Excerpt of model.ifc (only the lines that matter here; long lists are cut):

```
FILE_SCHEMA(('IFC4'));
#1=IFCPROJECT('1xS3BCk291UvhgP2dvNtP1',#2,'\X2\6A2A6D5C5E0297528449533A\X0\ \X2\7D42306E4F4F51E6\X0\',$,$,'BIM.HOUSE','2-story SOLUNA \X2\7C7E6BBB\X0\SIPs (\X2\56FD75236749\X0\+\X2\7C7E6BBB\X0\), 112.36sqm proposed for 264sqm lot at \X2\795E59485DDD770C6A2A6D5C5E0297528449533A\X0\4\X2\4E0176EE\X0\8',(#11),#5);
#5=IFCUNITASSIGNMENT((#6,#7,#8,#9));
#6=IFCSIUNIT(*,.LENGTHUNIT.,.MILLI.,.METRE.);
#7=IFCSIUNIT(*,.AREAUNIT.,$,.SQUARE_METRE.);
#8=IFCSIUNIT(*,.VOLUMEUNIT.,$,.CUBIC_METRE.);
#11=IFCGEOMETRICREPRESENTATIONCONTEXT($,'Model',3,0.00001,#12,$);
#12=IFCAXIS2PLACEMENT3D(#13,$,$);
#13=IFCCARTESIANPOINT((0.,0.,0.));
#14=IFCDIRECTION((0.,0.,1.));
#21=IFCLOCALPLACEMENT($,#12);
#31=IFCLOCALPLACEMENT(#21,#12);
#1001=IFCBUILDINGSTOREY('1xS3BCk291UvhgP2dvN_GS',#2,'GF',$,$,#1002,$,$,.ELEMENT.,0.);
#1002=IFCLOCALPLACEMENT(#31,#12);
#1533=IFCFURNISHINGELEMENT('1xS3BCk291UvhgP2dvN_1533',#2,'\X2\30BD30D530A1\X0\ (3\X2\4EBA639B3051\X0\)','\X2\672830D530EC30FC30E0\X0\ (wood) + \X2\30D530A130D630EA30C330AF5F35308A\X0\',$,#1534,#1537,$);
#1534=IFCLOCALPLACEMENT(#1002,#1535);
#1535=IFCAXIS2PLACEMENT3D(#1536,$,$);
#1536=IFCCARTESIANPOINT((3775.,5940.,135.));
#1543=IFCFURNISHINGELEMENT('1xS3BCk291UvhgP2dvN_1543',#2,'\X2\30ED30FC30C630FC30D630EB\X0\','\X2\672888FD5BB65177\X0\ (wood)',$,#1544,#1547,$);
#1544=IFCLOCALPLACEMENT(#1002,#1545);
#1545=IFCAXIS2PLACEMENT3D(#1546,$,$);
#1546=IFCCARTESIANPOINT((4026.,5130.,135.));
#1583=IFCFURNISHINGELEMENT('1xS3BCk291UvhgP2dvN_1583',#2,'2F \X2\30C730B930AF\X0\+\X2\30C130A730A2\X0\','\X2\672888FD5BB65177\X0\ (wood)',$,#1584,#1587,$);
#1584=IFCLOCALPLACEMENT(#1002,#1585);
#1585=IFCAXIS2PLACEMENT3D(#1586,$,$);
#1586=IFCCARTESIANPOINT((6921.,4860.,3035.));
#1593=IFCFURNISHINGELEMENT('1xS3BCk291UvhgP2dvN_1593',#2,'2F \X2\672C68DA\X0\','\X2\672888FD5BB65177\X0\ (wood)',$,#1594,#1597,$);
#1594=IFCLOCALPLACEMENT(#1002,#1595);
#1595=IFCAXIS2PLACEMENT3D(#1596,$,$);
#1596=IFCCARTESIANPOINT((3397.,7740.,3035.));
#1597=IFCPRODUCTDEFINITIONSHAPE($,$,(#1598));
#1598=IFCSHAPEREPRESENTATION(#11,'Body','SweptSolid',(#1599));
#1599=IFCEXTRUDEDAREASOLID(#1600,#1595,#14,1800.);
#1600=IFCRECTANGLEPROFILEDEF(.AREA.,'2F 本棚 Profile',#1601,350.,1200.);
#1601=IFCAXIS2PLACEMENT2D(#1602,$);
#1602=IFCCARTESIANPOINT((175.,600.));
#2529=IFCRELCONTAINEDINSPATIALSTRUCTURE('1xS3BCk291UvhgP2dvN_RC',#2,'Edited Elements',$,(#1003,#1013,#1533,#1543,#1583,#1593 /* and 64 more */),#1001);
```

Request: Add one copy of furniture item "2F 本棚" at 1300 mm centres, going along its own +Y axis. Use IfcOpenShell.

```python
import ifcopenshell
import ifcopenshell.api.geometry
import ifcopenshell.api.root
import ifcopenshell.util.element
import ifcopenshell.util.placement
import ifcopenshell.util.unit

model = ifcopenshell.open("model.ifc")
unit_scale = ifcopenshell.util.unit.calculate_unit_scale(model)


def reuse_history(source, copy):
    """copy_class also copies each property set's owner history, people and application; keep the originals."""
    for rel in copy.IsDefinedBy:
        if rel.is_a("IfcRelDefinesByProperties") and (history := rel.RelatingPropertyDefinition.OwnerHistory):
            rel.RelatingPropertyDefinition.OwnerHistory = source.OwnerHistory
            ifcopenshell.util.element.remove_deep2(model, history)


source = model.by_id(1593)
base = ifcopenshell.util.placement.get_local_placement(source.ObjectPlacement)
step = base[:3, 1] * 1.3 / unit_scale

for i in range(1, 2):
    copy = ifcopenshell.api.root.copy_class(model, product=source)
    copy.Representation = ifcopenshell.util.element.copy_deep(
        model, source.Representation, exclude=["IfcGeometricRepresentationContext", "IfcRepresentationMap"]
    )
    reuse_history(source, copy)
    matrix = base.copy()
    matrix[:3, 3] += i * step
    print("added at", matrix[:3, 3].round(3) + 0.0)
    ifcopenshell.api.geometry.edit_object_placement(model, product=copy, matrix=matrix, is_si=False)

model.write("model_v2.ifc")
```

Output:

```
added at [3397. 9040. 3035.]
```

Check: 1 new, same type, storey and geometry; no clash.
